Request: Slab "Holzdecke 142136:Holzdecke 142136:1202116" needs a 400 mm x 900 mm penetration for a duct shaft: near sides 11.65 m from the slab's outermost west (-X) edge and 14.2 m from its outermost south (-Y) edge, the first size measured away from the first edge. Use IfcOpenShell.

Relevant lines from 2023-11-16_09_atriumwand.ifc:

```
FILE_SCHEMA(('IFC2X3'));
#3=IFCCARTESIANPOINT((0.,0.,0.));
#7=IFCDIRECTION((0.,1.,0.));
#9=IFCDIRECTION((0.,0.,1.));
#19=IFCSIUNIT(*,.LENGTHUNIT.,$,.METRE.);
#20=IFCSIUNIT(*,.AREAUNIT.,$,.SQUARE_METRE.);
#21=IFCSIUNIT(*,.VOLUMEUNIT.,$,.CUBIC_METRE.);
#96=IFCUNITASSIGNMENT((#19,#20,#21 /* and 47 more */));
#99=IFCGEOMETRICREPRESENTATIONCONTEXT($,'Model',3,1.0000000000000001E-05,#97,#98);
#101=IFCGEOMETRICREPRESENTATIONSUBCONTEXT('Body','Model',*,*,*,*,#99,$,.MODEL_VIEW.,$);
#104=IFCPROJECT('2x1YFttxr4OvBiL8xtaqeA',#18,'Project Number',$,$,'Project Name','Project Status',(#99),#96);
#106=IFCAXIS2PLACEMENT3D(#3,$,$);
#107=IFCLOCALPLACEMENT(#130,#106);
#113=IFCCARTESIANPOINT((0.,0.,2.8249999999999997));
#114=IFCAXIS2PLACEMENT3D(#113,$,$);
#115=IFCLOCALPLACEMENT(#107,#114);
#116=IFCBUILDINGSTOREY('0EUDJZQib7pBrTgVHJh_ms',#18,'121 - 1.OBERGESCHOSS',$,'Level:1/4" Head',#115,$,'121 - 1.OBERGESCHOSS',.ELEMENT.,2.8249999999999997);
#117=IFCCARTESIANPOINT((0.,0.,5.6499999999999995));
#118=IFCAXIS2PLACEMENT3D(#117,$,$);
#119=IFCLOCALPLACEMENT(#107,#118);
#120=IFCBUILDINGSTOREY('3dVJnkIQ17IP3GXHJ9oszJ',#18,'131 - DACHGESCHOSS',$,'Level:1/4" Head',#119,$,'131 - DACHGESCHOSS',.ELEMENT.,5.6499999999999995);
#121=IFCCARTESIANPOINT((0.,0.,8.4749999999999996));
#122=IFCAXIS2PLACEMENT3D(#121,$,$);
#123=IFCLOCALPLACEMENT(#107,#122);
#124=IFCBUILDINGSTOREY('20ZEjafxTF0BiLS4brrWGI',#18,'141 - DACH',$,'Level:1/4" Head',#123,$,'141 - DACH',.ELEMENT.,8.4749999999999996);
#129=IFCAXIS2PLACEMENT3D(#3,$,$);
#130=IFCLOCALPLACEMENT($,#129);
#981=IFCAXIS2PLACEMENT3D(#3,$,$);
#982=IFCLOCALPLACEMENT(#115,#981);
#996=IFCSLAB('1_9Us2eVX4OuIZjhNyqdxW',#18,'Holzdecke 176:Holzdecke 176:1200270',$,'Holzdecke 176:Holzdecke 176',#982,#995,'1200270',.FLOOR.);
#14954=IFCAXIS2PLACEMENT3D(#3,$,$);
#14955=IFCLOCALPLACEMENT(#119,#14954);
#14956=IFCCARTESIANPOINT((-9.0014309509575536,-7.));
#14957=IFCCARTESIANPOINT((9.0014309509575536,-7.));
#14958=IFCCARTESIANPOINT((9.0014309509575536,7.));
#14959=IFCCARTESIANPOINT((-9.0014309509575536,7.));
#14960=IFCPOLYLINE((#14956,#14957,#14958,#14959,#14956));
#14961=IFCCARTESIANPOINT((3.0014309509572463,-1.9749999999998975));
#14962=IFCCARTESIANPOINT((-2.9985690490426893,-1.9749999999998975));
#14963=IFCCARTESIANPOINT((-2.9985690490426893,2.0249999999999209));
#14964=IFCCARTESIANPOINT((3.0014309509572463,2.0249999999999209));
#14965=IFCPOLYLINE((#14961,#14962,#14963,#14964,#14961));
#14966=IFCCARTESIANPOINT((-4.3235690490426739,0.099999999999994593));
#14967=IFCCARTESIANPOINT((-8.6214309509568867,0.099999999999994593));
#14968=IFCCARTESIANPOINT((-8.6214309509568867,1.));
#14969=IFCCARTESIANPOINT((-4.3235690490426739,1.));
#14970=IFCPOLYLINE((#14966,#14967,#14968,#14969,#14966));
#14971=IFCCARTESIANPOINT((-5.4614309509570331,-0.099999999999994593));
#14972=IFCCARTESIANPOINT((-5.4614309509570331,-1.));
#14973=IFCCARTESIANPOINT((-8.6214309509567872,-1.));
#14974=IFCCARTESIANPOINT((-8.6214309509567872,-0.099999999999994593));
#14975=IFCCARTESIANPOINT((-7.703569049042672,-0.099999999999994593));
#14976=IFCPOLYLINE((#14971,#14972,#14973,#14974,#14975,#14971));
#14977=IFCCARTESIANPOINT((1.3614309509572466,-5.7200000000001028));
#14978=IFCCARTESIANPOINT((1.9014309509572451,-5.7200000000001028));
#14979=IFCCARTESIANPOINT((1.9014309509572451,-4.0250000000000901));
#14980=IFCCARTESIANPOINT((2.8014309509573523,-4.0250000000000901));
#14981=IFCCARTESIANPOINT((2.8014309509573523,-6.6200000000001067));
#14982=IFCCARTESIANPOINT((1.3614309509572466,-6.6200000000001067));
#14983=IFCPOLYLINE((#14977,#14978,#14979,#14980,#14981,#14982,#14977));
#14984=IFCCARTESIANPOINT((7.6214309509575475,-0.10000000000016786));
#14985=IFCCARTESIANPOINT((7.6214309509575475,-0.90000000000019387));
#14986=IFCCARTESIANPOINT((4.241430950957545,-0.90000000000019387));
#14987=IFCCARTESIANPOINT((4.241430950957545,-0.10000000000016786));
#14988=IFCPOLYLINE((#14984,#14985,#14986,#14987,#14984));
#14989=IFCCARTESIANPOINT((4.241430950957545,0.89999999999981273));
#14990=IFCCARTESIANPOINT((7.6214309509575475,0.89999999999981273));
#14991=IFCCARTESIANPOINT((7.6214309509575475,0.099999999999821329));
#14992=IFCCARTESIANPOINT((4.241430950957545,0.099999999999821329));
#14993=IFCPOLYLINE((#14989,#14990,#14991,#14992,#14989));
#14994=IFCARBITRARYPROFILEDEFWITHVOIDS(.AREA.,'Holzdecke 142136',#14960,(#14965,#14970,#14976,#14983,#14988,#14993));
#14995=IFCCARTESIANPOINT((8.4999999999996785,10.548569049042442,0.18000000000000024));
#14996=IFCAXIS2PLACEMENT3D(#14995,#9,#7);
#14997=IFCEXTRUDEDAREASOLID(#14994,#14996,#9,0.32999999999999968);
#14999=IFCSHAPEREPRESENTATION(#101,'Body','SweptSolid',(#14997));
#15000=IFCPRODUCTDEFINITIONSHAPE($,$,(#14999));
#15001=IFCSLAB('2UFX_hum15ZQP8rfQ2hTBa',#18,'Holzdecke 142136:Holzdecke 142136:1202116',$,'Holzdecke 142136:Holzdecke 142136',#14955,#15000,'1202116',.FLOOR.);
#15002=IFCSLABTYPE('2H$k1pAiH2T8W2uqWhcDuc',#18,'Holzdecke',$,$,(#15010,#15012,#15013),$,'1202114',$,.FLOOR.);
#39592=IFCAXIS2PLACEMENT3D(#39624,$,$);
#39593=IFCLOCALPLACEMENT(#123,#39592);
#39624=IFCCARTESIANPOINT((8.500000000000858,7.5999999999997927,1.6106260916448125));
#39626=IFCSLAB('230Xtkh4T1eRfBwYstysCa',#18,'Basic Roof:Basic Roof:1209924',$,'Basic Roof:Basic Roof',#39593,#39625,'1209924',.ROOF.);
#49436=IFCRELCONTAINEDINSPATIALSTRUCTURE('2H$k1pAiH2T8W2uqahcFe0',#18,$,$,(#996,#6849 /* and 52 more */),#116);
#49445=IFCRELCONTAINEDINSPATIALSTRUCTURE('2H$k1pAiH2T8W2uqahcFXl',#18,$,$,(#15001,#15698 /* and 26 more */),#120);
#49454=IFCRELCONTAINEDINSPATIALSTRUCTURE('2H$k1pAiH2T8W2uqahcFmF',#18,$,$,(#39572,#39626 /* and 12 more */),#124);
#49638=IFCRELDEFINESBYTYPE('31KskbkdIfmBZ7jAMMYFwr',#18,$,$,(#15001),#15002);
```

```python
import numpy as np
import ifcopenshell
import ifcopenshell.api.feature
import ifcopenshell.api.geometry
import ifcopenshell.api.root
import ifcopenshell.geom
import ifcopenshell.util.placement
import ifcopenshell.util.representation
import ifcopenshell.util.shape
import ifcopenshell.util.unit

model = ifcopenshell.open("2023-11-16_09_atriumwand.ifc")
unit_scale = ifcopenshell.util.unit.calculate_unit_scale(model)
settings = ifcopenshell.geom.settings()


def volume(element):
    """Net volume in cubic metres, openings subtracted."""
    shape = ifcopenshell.geom.create_shape(settings, element)
    return ifcopenshell.util.shape.get_volume(shape.geometry)


slab = model.by_id(15001)
before = volume(slab)

# Extent in the slab's own axes, in metres. The edges named are its -X and -Y sides.
slab_shape = ifcopenshell.geom.create_shape(settings, slab)
vertices = ifcopenshell.util.shape.get_vertices(slab_shape.geometry)
x_min, y_min, bottom = vertices.min(axis=0)
top = vertices[:, 2].max()

opening = ifcopenshell.api.root.create_entity(model, ifc_class="IfcOpeningElement", name="Duct shaft opening")
context = ifcopenshell.util.representation.get_context(model, "Model", "Body", "MODEL_VIEW")
width, depth = 0.4, 0.9
outline = [(0.0, 0.0), (width, 0.0), (width, depth), (0.0, depth), (0.0, 0.0)]
# Overshoot both faces by 50 mm so the cut is clean.
shape = ifcopenshell.api.geometry.add_slab_representation(
    model, context=context, depth=top - bottom + 0.1, polyline=outline
)
ifcopenshell.api.geometry.assign_representation(model, product=opening, representation=shape)

matrix = ifcopenshell.util.placement.get_local_placement(slab.ObjectPlacement)
matrix[:, 3] = matrix @ np.append(np.array([x_min + 11.65, y_min + 14.2, bottom - 0.05]) / unit_scale, 1.0)
ifcopenshell.api.geometry.edit_object_placement(model, product=opening, matrix=matrix, is_si=False)
ifcopenshell.api.feature.add_feature(model, feature=opening, element=slab)

after = volume(slab)

print(f"slab volume {before:.3f} -> {after:.3f} m3")

model.write("2023-11-16_09_atriumwand_v2.ifc")
```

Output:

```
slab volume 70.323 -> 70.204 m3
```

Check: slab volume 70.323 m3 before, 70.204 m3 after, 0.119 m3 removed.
